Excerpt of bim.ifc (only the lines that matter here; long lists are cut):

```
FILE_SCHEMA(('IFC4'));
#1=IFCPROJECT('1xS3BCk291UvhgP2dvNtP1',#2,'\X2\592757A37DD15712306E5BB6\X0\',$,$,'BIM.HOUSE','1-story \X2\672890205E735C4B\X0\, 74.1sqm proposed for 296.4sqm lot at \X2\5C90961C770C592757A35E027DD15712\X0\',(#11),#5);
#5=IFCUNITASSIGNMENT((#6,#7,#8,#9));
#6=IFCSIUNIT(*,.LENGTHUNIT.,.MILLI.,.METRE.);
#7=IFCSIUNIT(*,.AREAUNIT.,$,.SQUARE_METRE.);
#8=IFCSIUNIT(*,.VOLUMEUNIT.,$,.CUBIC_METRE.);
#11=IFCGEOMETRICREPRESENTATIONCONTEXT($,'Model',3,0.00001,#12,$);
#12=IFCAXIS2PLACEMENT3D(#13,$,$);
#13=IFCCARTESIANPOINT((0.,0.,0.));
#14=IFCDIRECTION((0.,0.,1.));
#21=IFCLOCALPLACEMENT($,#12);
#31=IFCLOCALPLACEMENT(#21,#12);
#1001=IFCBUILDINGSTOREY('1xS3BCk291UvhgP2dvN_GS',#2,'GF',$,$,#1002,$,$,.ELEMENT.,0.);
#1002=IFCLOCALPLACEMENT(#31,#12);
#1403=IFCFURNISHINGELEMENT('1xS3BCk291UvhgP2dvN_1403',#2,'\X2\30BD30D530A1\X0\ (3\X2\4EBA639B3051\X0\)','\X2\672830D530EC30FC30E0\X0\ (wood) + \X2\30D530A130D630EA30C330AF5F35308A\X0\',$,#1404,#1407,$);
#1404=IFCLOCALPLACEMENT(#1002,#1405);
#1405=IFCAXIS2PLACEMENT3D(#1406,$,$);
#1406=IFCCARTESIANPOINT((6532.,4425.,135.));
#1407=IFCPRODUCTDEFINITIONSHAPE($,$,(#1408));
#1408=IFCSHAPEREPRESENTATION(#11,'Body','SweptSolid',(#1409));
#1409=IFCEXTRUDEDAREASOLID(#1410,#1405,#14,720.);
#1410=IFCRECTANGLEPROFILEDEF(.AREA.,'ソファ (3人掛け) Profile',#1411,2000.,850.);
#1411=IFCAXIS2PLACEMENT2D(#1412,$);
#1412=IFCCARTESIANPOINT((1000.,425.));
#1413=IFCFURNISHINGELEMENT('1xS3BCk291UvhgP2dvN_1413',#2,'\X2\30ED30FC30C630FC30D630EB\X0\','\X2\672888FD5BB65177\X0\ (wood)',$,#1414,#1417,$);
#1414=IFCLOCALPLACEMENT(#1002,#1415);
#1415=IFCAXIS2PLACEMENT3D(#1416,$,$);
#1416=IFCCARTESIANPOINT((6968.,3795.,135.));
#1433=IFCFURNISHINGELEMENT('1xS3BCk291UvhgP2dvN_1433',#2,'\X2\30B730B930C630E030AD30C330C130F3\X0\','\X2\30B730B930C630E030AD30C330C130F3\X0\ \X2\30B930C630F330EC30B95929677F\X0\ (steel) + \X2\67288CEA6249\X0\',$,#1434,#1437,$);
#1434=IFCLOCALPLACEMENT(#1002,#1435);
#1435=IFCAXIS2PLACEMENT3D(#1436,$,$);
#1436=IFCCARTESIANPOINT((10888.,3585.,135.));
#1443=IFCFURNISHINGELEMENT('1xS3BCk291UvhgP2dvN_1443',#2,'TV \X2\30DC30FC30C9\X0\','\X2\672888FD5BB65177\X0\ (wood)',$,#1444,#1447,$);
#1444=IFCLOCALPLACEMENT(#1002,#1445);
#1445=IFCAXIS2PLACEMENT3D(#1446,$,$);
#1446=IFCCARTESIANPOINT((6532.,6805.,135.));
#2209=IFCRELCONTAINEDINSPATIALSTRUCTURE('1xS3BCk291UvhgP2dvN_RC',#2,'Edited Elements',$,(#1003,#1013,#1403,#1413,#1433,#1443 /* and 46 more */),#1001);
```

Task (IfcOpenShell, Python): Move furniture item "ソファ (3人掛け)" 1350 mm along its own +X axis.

```python
import ifcopenshell
import ifcopenshell.api.geometry
import ifcopenshell.util.placement
import ifcopenshell.util.unit

model = ifcopenshell.open("bim.ifc")
unit_scale = ifcopenshell.util.unit.calculate_unit_scale(model)

item = model.by_guid("1xS3BCk291UvhgP2dvN_1403")
matrix = ifcopenshell.util.placement.get_local_placement(item.ObjectPlacement)
matrix[:3, 3] += matrix[:3, 0] * 1.35 / unit_scale
ifcopenshell.api.geometry.edit_object_placement(model, product=item, matrix=matrix, is_si=False)

print(ifcopenshell.util.placement.get_local_placement(item.ObjectPlacement).round(3) + 0.0)

model.write("bim_rev.ifc")
```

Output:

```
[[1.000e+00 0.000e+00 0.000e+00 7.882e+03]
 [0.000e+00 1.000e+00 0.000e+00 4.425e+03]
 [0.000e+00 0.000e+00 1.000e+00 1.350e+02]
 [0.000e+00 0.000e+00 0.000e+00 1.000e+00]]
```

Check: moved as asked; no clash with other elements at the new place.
